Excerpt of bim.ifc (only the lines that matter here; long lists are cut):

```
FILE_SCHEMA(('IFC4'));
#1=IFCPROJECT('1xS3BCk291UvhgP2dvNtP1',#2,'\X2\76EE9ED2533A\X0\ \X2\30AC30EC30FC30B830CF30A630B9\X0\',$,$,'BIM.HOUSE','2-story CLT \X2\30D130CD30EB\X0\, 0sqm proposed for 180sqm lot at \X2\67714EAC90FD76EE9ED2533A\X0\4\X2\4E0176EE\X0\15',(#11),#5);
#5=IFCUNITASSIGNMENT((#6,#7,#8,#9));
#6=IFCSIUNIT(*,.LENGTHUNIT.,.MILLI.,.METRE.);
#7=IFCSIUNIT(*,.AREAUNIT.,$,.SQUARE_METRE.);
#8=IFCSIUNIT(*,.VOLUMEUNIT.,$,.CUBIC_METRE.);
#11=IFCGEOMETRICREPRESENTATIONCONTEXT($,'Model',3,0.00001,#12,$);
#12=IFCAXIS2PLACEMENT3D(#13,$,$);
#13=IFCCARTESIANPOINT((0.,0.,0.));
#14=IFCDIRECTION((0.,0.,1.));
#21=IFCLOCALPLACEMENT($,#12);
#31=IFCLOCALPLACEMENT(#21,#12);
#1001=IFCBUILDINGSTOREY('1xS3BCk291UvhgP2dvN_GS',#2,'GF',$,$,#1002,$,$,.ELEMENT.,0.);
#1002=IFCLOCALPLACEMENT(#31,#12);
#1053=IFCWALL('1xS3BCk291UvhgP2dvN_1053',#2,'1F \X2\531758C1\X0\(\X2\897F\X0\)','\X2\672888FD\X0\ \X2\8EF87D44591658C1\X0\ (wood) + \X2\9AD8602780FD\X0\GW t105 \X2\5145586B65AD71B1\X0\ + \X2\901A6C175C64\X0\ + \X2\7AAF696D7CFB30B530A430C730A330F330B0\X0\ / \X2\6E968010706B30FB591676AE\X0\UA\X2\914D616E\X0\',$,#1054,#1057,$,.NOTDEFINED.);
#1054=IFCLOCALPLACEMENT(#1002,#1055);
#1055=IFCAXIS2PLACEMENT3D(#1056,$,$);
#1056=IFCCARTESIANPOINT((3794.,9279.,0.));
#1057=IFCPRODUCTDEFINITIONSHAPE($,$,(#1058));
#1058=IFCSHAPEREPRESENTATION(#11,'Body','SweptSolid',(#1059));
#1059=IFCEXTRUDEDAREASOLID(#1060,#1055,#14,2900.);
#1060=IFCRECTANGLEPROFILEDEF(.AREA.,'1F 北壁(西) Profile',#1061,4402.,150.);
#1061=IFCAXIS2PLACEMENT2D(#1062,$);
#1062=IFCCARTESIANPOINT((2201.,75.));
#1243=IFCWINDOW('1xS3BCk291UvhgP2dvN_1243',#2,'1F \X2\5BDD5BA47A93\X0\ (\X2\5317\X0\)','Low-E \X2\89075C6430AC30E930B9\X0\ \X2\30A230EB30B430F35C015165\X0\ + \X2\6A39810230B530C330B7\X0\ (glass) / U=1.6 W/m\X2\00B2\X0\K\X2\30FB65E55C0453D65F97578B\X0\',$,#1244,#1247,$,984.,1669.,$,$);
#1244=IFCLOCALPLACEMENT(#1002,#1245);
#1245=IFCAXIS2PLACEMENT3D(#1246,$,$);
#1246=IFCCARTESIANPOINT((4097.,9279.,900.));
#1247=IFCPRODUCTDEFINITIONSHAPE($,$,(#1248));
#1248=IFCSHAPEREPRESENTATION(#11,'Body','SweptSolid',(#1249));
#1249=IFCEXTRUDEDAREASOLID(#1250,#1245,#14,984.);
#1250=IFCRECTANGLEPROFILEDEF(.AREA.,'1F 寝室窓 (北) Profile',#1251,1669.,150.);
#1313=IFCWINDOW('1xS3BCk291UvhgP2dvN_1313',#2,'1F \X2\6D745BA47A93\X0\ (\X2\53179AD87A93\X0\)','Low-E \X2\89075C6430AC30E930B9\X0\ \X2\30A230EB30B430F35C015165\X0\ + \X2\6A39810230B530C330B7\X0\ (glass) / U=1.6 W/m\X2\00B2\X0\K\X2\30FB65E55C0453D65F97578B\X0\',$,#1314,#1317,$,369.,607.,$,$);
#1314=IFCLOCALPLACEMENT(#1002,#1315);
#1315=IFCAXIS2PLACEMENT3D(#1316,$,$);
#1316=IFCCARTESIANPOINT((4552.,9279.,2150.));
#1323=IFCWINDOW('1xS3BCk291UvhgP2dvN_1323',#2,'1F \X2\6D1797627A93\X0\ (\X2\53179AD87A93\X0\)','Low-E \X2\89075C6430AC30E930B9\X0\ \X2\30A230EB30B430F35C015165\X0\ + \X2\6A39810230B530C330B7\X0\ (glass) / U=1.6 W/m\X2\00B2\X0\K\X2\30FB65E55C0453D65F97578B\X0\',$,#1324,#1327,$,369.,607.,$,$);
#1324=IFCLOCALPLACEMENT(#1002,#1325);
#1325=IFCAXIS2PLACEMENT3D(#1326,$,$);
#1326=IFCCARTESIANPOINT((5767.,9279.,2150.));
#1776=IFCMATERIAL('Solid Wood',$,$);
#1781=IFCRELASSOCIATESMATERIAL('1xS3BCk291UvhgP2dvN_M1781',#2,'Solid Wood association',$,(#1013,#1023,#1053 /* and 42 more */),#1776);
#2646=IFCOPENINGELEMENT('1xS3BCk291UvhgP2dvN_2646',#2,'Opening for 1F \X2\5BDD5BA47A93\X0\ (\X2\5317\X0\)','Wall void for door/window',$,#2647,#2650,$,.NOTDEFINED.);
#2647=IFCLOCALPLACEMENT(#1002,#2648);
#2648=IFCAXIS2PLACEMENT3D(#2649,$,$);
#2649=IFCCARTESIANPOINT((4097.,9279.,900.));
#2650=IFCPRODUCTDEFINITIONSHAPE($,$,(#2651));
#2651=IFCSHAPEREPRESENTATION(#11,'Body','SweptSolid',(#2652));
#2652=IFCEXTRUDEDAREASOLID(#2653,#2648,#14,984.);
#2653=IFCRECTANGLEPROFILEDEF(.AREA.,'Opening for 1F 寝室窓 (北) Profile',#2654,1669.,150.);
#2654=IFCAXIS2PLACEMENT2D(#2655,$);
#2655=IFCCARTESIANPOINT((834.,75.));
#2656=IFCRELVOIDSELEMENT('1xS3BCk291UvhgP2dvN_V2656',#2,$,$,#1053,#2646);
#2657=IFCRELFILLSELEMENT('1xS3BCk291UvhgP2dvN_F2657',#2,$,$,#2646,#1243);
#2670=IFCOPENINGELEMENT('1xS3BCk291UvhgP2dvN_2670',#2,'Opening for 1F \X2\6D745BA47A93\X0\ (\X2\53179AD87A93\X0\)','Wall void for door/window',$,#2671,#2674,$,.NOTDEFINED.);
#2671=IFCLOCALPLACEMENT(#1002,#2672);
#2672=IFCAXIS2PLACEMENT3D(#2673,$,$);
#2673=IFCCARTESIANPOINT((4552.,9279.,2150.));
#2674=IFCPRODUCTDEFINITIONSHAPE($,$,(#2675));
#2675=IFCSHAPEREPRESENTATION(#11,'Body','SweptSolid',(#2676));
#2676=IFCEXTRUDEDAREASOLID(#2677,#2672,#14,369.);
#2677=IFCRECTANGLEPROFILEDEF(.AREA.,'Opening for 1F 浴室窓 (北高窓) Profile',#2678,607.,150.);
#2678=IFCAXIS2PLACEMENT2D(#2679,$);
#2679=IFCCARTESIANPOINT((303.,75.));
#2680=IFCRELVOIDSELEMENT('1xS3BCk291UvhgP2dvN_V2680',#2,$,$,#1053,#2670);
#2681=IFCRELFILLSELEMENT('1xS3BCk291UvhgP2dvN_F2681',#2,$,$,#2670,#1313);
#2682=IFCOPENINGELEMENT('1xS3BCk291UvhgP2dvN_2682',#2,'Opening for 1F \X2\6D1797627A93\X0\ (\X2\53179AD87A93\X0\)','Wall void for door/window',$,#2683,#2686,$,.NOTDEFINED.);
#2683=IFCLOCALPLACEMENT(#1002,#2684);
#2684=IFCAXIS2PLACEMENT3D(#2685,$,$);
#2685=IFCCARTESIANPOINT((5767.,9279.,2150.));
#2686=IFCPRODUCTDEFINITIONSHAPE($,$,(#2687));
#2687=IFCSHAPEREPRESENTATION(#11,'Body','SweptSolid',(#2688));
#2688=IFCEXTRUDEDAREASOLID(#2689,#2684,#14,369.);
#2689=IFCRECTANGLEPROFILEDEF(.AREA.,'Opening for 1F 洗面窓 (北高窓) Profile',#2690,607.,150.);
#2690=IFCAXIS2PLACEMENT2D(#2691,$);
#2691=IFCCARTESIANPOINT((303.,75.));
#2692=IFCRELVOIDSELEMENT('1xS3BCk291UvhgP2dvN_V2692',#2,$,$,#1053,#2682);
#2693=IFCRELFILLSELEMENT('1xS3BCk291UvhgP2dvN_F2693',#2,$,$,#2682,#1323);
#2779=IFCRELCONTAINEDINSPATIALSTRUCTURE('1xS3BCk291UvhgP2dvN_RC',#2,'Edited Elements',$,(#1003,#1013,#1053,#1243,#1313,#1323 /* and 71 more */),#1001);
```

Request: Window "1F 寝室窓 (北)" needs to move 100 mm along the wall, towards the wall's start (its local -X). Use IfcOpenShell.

```python
import ifcopenshell
import ifcopenshell.api.geometry
import ifcopenshell.util.placement
import ifcopenshell.util.unit

model = ifcopenshell.open("bim.ifc")
unit_scale = ifcopenshell.util.unit.calculate_unit_scale(model)

window = model.by_guid("1xS3BCk291UvhgP2dvN_1243")
opening = window.FillsVoids[0].RelatingOpeningElement
wall = opening.VoidsElements[0].RelatingBuildingElement

wall_matrix = ifcopenshell.util.placement.get_local_placement(wall.ObjectPlacement)
shift = wall_matrix[:3, 0] * -0.1 / unit_scale
before = ifcopenshell.util.placement.get_local_placement(window.ObjectPlacement)[:3, 3].copy()

# The window is not placed relative to its opening, so move both.
for product in (opening, window):
    matrix = ifcopenshell.util.placement.get_local_placement(product.ObjectPlacement)
    matrix[:3, 3] += shift
    ifcopenshell.api.geometry.edit_object_placement(model, product=product, matrix=matrix, is_si=False)

after = ifcopenshell.util.placement.get_local_placement(window.ObjectPlacement)[:3, 3]
print("window moved by", (after - before).round(3) + 0.0)

model.write("bim_v2.ifc")
```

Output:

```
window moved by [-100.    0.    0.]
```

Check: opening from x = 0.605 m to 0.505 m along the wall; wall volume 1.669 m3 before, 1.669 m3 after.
